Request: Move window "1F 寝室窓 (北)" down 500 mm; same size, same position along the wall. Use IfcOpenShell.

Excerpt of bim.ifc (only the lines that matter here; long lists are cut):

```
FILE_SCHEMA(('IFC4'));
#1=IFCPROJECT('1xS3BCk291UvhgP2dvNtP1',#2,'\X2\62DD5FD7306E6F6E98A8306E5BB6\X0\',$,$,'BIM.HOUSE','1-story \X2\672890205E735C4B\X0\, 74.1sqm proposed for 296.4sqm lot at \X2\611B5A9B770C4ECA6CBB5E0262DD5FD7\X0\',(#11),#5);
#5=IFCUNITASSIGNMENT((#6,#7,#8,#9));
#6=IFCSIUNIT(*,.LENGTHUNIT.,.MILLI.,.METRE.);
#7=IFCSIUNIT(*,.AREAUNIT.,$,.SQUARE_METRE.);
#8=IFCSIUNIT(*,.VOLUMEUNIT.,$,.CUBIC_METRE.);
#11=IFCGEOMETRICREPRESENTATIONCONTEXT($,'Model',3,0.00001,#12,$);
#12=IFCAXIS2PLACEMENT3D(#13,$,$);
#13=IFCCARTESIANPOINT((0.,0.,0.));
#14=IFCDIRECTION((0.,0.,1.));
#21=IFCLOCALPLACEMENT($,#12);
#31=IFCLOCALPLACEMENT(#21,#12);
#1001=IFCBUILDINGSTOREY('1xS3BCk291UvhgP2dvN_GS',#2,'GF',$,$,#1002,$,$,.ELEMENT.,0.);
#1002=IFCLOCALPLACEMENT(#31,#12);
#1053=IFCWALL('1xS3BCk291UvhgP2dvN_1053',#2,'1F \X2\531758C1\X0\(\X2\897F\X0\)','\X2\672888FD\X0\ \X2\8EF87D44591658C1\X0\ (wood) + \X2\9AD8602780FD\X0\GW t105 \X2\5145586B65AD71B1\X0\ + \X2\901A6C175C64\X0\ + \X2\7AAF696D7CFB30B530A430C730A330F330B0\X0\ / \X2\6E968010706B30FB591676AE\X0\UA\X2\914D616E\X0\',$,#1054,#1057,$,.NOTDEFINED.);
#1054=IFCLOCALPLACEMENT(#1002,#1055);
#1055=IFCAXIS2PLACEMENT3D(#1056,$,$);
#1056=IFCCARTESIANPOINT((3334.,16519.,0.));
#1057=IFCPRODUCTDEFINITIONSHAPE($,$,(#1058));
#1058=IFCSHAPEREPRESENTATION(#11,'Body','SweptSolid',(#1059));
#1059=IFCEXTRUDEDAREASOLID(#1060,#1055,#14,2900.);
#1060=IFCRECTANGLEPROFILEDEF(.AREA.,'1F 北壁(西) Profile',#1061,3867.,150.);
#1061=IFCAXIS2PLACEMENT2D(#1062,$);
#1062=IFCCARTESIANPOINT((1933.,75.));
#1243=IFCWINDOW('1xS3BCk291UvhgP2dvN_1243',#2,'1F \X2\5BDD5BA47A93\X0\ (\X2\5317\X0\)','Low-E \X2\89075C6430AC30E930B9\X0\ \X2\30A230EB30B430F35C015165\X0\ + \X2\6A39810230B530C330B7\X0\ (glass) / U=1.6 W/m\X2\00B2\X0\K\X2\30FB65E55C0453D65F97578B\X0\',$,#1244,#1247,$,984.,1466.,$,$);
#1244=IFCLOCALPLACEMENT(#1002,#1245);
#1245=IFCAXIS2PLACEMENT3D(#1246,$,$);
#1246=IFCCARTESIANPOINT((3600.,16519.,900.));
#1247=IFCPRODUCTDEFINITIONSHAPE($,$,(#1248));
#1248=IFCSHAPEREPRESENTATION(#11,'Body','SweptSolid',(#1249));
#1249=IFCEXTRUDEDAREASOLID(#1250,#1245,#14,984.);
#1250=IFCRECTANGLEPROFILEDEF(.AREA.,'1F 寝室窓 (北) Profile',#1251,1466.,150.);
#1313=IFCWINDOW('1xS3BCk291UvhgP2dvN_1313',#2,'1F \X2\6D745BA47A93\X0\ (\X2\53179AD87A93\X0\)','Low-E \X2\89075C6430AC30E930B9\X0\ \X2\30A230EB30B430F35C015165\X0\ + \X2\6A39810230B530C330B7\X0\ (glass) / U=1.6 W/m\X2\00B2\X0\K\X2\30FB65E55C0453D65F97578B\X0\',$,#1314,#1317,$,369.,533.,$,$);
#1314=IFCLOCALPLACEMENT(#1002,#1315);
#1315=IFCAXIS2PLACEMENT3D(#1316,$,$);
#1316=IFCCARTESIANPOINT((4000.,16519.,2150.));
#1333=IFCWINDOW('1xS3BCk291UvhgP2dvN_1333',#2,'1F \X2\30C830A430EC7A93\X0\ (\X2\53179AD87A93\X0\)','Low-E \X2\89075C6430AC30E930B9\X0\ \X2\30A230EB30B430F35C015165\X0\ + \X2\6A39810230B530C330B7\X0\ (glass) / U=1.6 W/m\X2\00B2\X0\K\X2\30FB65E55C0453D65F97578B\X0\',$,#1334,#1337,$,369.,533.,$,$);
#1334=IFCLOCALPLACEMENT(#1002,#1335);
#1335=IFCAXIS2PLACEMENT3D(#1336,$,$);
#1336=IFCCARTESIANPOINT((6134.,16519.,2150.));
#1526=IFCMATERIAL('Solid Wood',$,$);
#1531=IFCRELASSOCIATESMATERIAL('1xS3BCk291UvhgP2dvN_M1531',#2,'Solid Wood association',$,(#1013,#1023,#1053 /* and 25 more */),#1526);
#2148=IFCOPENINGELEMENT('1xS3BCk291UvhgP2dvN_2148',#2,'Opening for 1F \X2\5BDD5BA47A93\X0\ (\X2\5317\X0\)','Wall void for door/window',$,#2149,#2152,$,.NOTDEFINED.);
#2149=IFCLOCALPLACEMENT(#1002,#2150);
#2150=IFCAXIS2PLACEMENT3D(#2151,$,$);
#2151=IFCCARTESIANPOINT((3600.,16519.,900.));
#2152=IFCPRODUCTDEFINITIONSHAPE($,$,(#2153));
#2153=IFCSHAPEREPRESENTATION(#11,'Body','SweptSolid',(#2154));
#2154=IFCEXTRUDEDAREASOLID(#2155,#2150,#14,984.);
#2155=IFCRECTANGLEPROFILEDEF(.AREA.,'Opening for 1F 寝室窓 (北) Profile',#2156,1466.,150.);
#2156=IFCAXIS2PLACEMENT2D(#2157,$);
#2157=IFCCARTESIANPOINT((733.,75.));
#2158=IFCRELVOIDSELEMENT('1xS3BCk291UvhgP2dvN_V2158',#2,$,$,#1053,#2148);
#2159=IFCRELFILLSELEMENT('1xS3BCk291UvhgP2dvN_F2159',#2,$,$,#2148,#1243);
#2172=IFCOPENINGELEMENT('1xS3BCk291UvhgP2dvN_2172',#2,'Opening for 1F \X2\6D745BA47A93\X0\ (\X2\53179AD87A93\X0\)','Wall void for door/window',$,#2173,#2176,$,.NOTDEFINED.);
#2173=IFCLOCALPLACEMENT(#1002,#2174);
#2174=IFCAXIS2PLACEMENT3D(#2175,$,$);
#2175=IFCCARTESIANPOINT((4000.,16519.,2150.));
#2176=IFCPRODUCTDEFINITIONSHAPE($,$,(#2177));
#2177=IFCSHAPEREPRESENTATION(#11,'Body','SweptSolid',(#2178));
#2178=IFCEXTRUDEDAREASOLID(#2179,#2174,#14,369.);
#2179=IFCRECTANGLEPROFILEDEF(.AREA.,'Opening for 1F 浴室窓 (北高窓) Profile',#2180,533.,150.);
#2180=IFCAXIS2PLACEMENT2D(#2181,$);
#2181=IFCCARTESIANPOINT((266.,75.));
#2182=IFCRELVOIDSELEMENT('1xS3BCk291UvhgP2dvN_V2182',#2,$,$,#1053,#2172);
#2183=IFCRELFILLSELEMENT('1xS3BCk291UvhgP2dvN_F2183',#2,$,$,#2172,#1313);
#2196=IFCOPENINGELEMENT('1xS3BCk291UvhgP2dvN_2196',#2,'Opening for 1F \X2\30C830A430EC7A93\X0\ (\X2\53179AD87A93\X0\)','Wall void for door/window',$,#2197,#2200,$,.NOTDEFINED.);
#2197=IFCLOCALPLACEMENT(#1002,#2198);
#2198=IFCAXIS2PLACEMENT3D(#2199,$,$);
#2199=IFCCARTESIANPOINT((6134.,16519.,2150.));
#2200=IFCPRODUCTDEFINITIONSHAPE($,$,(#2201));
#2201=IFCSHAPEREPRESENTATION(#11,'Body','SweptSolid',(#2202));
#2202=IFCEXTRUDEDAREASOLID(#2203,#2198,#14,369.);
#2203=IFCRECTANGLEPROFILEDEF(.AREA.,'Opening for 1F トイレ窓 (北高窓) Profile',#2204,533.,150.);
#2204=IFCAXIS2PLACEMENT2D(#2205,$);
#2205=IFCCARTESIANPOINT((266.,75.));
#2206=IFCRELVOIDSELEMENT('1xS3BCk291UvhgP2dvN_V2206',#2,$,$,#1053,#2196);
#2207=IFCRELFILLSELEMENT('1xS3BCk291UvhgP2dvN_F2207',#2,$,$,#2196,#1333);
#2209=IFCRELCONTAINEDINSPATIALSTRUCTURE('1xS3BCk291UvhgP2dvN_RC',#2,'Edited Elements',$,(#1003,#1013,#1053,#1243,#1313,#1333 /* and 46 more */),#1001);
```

```python
import numpy as np
import ifcopenshell
import ifcopenshell.api.geometry
import ifcopenshell.util.placement
import ifcopenshell.util.unit

model = ifcopenshell.open("bim.ifc")
unit_scale = ifcopenshell.util.unit.calculate_unit_scale(model)

window = model.by_id(1243)
opening = window.FillsVoids[0].RelatingOpeningElement
dz = -500.0

shift = np.array([0.0, 0.0, dz])
# The window is not placed relative to its opening, so move both.
for product in (opening, window):
    matrix = ifcopenshell.util.placement.get_local_placement(product.ObjectPlacement)
    matrix[:3, 3] += shift
    ifcopenshell.api.geometry.edit_object_placement(model, product=product, matrix=matrix, is_si=False)

print(f"moved by {dz * unit_scale:+.3f} m")

model.write("bim_updated.ifc")
```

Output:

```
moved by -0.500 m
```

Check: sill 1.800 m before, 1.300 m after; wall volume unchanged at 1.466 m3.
